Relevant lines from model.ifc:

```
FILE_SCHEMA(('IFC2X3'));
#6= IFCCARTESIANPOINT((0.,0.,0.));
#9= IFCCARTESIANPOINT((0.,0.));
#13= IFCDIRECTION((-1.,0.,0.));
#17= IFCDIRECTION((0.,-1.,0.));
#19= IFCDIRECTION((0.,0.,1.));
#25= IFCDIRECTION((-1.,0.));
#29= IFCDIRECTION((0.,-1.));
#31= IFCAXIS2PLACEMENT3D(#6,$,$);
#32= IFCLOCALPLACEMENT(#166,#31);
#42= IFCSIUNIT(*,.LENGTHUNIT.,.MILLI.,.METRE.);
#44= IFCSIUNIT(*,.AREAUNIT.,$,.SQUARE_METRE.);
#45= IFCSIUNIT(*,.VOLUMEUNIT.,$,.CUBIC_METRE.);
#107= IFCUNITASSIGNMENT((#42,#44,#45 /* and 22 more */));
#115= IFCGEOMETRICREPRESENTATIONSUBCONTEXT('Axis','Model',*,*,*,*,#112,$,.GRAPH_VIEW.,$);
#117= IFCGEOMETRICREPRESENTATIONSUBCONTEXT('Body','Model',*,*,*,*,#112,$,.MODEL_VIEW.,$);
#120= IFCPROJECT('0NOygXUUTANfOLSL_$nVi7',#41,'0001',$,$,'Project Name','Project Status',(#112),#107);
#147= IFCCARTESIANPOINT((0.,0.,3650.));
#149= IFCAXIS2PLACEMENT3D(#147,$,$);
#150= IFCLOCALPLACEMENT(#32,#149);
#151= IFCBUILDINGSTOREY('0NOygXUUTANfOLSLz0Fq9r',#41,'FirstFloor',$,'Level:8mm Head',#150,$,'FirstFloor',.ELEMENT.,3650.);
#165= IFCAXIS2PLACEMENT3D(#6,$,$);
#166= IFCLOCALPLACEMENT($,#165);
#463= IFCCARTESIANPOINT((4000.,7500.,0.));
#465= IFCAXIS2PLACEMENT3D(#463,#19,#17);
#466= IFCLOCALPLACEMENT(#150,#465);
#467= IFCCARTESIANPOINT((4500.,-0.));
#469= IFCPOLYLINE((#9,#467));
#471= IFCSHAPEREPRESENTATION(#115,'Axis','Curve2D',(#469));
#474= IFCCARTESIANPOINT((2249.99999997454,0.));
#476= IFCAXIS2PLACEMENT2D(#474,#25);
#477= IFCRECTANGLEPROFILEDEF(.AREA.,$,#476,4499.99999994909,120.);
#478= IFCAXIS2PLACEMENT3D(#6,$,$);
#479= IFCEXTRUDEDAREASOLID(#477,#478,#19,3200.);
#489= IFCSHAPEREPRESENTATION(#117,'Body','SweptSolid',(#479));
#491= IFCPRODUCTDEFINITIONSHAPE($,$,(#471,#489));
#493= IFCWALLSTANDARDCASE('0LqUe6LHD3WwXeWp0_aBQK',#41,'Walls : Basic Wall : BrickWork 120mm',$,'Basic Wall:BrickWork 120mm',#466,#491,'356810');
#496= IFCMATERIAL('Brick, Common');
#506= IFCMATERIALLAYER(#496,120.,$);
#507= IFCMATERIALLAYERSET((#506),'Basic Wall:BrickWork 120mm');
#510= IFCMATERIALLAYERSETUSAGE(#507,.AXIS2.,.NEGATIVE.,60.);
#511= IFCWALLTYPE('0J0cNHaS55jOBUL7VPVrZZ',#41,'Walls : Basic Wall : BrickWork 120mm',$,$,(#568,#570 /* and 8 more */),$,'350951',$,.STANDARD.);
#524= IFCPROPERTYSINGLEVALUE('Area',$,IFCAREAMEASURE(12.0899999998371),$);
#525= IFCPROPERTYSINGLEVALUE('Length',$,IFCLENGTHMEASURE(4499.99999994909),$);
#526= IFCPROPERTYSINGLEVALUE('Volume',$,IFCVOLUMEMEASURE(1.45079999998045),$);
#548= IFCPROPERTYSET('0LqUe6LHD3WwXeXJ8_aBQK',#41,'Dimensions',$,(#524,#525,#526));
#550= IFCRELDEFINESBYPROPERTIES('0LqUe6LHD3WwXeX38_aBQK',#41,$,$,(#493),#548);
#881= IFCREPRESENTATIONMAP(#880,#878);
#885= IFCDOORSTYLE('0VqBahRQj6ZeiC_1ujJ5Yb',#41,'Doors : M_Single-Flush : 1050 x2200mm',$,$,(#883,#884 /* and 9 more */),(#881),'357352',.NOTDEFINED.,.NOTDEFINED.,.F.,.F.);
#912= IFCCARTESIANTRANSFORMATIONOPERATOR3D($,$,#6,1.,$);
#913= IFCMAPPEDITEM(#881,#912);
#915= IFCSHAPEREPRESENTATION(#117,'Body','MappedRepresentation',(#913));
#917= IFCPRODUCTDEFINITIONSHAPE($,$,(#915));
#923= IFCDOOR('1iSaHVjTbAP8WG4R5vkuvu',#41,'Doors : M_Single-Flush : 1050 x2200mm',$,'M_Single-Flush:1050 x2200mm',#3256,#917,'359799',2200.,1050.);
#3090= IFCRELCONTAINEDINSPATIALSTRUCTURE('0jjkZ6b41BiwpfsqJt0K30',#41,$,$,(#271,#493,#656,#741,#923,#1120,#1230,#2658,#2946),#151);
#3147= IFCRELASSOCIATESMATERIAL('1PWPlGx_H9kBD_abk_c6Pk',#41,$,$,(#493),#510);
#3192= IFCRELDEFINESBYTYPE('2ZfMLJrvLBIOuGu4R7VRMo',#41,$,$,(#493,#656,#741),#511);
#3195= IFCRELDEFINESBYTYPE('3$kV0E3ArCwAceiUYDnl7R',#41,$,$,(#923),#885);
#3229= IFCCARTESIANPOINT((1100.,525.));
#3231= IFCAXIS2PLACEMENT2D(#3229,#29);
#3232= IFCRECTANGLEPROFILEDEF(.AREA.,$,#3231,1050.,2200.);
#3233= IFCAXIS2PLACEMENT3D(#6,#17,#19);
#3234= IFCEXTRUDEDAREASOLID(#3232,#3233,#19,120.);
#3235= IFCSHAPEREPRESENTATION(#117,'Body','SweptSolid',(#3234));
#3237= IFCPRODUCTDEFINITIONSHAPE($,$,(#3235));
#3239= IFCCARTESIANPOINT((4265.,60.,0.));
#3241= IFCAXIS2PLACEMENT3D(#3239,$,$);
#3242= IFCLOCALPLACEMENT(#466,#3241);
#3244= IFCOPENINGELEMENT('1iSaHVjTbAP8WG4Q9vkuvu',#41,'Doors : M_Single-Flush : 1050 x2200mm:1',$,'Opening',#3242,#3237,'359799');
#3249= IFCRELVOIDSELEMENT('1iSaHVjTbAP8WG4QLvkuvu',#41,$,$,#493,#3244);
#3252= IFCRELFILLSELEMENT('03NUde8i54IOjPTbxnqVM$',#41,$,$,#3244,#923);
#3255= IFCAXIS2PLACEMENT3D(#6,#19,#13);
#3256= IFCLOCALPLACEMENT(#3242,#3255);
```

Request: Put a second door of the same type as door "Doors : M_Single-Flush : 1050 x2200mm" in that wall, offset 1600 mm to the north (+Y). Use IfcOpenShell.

```python
import ifcopenshell
import ifcopenshell.api.feature
import ifcopenshell.api.geometry
import ifcopenshell.api.pset
import ifcopenshell.api.root
import ifcopenshell.geom
import ifcopenshell.util.element
import ifcopenshell.util.placement
import ifcopenshell.util.shape
import ifcopenshell.util.unit

model = ifcopenshell.open("model.ifc")
unit_scale = ifcopenshell.util.unit.calculate_unit_scale(model)
area_scale = ifcopenshell.util.unit.calculate_unit_scale(model, "AREAUNIT")
volume_scale = ifcopenshell.util.unit.calculate_unit_scale(model, "VOLUMEUNIT")
settings = ifcopenshell.geom.settings()


def volume(element):
    """Net volume in cubic metres, openings subtracted."""
    shape = ifcopenshell.geom.create_shape(settings, element)
    return ifcopenshell.util.shape.get_volume(shape.geometry)


def reuse_history(source, copy):
    """copy_class also copies each property set's owner history, people and application; keep the originals."""
    for rel in copy.IsDefinedBy:
        if rel.is_a("IfcRelDefinesByProperties") and (history := rel.RelatingPropertyDefinition.OwnerHistory):
            rel.RelatingPropertyDefinition.OwnerHistory = source.OwnerHistory
            ifcopenshell.util.element.remove_deep2(model, history)


door = model.by_guid("1iSaHVjTbAP8WG4R5vkuvu")
opening = door.FillsVoids[0].RelatingOpeningElement
wall = opening.VoidsElements[0].RelatingBuildingElement
before = volume(wall)
shift = ifcopenshell.util.placement.get_local_placement(wall.ObjectPlacement)[:3, 0] * -1.6 / unit_scale

# copy_class copies the void relationship, type, container and properties, but no geometry.
new_opening = ifcopenshell.api.root.copy_class(model, product=opening)
new_opening.Representation = ifcopenshell.util.element.copy_deep(
    model, opening.Representation, exclude=["IfcGeometricRepresentationContext", "IfcRepresentationMap"]
)
new_opening.Tag = None
new_door = ifcopenshell.api.root.copy_class(model, product=door)
new_door.Representation = ifcopenshell.util.element.copy_deep(
    model, door.Representation, exclude=["IfcGeometricRepresentationContext", "IfcRepresentationMap"]
)
new_door.Tag = None
reuse_history(door, new_door)
fills = ifcopenshell.api.feature.add_filling(model, opening=new_opening, element=new_door)
fills.OwnerHistory = new_door.OwnerHistory  # required in IFC2X3

for old, new in ((opening, new_opening), (door, new_door)):
    matrix = ifcopenshell.util.placement.get_local_placement(old.ObjectPlacement)
    matrix[:3, 3] += shift
    ifcopenshell.api.geometry.edit_object_placement(model, product=new, matrix=matrix, is_si=False)

after = volume(wall)
thickness = 0.12  # wall thickness in metres

# Update the wall's stored quantities.
pset = model.by_id(ifcopenshell.util.element.get_pset(wall, "Dimensions", should_inherit=False)["id"])
ifcopenshell.api.pset.edit_pset(model, pset=pset, properties={
    "Area": model.create_entity("IfcAreaMeasure", after / thickness / area_scale),
    "Volume": model.create_entity("IfcVolumeMeasure", after / volume_scale),
})

print(f"wall volume {before:.3f} -> {after:.3f} m3")

model.write("model_v2.ifc")
```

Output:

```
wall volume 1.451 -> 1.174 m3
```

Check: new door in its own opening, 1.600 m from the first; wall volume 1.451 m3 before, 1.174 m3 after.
